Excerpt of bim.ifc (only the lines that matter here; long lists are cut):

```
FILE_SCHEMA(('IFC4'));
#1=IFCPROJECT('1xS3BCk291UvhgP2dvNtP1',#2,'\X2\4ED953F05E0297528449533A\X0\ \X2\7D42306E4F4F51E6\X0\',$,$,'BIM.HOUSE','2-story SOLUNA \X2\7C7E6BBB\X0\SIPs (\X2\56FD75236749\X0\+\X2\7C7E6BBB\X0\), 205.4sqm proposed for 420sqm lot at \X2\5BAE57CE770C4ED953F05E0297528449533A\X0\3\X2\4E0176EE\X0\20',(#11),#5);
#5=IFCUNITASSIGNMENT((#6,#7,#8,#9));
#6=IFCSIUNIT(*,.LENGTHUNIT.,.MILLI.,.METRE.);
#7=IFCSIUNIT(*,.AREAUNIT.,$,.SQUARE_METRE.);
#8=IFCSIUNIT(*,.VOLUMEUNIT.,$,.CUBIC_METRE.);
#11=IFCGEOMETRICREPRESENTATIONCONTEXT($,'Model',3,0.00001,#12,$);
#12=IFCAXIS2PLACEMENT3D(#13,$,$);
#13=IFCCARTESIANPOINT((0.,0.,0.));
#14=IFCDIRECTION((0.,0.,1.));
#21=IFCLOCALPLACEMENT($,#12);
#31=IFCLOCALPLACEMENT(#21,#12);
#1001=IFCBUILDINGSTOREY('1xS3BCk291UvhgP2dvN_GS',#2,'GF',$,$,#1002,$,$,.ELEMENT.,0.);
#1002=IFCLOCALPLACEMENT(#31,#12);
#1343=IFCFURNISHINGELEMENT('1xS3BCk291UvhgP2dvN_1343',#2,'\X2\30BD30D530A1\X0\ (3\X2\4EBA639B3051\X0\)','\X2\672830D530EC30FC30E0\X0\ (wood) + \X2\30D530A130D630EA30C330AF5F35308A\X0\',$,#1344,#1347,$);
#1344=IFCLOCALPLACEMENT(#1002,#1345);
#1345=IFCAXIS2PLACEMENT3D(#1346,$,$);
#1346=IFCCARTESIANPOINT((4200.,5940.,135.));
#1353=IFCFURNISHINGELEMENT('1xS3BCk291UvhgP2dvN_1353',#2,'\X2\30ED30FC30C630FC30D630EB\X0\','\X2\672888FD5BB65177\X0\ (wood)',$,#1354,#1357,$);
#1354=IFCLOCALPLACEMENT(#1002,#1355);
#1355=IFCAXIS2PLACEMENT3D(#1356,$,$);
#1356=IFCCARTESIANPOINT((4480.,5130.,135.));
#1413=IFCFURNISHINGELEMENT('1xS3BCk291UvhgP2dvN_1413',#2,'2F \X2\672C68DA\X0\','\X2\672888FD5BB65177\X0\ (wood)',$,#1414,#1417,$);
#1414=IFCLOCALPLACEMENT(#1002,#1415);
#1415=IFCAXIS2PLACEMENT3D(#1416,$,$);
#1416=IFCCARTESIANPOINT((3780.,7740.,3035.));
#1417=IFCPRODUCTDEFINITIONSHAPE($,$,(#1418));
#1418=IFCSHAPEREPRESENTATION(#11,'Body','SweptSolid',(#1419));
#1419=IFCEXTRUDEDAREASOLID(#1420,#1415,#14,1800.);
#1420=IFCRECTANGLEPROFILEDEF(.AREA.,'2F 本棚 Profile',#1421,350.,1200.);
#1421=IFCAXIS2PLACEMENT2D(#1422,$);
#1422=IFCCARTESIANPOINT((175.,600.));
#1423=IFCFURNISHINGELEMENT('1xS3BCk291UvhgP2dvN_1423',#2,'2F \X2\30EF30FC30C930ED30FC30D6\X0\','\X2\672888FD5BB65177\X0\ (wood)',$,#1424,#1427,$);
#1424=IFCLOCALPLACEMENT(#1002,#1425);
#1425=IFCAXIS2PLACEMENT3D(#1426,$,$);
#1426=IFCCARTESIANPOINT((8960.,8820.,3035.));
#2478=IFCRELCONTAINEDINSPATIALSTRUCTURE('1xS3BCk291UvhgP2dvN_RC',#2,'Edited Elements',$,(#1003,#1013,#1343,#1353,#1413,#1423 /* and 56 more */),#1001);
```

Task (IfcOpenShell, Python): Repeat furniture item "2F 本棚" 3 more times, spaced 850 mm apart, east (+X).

```python
import numpy as np
import ifcopenshell
import ifcopenshell.api.geometry
import ifcopenshell.api.root
import ifcopenshell.util.element
import ifcopenshell.util.placement
import ifcopenshell.util.unit

model = ifcopenshell.open("bim.ifc")
unit_scale = ifcopenshell.util.unit.calculate_unit_scale(model)


def reuse_history(source, copy):
    """copy_class also copies each property set's owner history, people and application; keep the originals."""
    for rel in copy.IsDefinedBy:
        if rel.is_a("IfcRelDefinesByProperties") and (history := rel.RelatingPropertyDefinition.OwnerHistory):
            rel.RelatingPropertyDefinition.OwnerHistory = source.OwnerHistory
            ifcopenshell.util.element.remove_deep2(model, history)


source = model.by_guid("1xS3BCk291UvhgP2dvN_1413")
base = ifcopenshell.util.placement.get_local_placement(source.ObjectPlacement)
step = np.array([1.0, 0.0, 0.0]) * 0.85 / unit_scale

for i in range(1, 4):
    copy = ifcopenshell.api.root.copy_class(model, product=source)
    copy.Representation = ifcopenshell.util.element.copy_deep(
        model, source.Representation, exclude=["IfcGeometricRepresentationContext", "IfcRepresentationMap"]
    )
    reuse_history(source, copy)
    matrix = base.copy()
    matrix[:3, 3] += i * step
    print("added at", matrix[:3, 3].round(3) + 0.0)
    ifcopenshell.api.geometry.edit_object_placement(model, product=copy, matrix=matrix, is_si=False)

model.write("bim-out.ifc")
```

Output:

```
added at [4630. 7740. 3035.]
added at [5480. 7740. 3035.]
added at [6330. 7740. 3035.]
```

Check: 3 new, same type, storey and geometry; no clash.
